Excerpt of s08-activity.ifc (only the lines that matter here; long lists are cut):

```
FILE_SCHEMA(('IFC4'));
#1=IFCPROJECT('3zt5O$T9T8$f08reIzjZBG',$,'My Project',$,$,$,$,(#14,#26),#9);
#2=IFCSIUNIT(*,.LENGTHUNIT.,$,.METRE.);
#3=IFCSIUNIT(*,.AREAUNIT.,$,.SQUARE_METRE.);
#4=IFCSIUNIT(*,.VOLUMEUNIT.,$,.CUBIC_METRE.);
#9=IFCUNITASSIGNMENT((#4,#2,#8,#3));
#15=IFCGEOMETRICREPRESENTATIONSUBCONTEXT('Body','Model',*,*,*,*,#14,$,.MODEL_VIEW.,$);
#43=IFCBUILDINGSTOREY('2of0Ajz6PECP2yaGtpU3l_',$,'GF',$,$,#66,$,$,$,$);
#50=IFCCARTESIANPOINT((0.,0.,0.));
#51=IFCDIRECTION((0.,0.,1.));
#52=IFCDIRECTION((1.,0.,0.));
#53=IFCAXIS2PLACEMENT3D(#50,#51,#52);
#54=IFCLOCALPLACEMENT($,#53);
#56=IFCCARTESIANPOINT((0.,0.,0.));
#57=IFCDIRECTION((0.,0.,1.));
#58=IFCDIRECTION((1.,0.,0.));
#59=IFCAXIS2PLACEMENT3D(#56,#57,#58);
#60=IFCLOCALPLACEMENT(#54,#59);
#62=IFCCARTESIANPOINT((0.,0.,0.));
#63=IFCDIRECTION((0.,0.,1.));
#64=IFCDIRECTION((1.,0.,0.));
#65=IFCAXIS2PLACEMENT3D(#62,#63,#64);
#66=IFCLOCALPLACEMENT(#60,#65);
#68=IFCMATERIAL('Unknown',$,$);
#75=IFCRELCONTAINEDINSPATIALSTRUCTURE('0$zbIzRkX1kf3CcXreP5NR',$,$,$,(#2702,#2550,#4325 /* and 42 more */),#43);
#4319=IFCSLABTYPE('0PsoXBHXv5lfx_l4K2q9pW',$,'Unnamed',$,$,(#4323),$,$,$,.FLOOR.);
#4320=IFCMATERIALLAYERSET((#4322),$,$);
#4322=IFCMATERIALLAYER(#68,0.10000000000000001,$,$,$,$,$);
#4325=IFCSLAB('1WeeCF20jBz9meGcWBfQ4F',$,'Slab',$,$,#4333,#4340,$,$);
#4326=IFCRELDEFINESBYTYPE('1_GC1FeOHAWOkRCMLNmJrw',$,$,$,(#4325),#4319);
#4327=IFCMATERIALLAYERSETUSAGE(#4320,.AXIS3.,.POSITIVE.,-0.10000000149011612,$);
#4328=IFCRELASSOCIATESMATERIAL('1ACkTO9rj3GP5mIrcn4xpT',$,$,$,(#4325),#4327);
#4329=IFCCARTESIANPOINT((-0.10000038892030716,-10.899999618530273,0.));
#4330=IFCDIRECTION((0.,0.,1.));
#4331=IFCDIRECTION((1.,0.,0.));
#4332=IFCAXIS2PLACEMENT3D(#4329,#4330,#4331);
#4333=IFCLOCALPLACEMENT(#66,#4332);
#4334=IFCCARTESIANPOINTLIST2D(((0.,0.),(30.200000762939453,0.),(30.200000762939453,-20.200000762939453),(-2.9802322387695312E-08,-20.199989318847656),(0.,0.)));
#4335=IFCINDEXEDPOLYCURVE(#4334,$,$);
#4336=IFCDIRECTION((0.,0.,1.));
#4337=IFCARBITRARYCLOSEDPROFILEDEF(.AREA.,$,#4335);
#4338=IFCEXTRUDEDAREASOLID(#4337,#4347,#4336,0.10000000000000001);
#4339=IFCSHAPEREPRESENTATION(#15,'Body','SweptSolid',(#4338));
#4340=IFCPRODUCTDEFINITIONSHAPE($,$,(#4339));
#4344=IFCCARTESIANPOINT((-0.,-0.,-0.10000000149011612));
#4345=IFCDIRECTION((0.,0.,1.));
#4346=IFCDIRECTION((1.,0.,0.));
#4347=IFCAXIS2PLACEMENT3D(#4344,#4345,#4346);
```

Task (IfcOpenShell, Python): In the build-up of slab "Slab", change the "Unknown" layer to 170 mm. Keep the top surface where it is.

```python
import ifcopenshell
import ifcopenshell.util.element
import ifcopenshell.util.representation
import ifcopenshell.util.unit

model = ifcopenshell.open("s08-activity.ifc")
unit_scale = ifcopenshell.util.unit.calculate_unit_scale(model)

layer_set = model.by_id(4320)
layer = next(l for l in layer_set.MaterialLayers if l.Material and l.Material.Name == "Unknown")
change = 0.17 / unit_scale - layer.LayerThickness
layer.LayerThickness += change

# Geometry does not follow the layer set by itself.
slabs = [e for e in ifcopenshell.util.element.get_elements_by_material(model, layer_set) if e.is_a("IfcSlab")]
for slab in sorted(slabs, key=lambda e: e.id()):
    body = ifcopenshell.util.representation.get_representation(slab, "Model", "Body")
    solid = body.Items[0]
    old_depth = solid.Depth
    solid.Depth += change
    # Extruded upwards: lower the start of the extrusion so the top stays.
    x, y, z = solid.Position.Location.Coordinates
    solid.Position.Location = model.createIfcCartesianPoint((x, y, z - change))
    print(slab.id(), f"{old_depth:g} -> {solid.Depth:g}")

# The layers are counted up from the underside, which has moved.
for usage in {ifcopenshell.util.element.get_material(slab) for slab in slabs}:
    usage.OffsetFromReferenceLine -= change

model.write("s08-activity_rev.ifc")
```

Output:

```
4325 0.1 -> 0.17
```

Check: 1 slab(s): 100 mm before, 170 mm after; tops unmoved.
